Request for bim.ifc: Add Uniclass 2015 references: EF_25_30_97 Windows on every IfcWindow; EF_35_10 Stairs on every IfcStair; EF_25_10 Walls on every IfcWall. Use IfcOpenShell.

First a look at what the model holds.

```python
import ifcopenshell

model = ifcopenshell.open("bim.ifc")
print(model.schema)
print("classifications:", [c.Name for c in model.by_type("IfcClassification")])
for ifc_class in ("IfcDoor", "IfcRoof", "IfcStair", "IfcWall", "IfcWindow"):
    print(ifc_class, len(model.by_type(ifc_class)))
```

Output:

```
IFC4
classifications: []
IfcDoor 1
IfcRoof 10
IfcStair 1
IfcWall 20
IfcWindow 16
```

```python
import ifcopenshell
import ifcopenshell.api.classification

model = ifcopenshell.open("bim.ifc")

system = ifcopenshell.api.classification.add_classification(model, classification="Uniclass 2015")

codes = {
    "IfcWindow": ("EF_25_30_97", "Windows"),
    "IfcStair": ("EF_35_10", "Stairs"),
    "IfcWall": ("EF_25_10", "Walls"),
}
for ifc_class, (code, name) in codes.items():
    products = model.by_type(ifc_class)
    ifcopenshell.api.classification.add_reference(
        model, products=products, classification=system, identification=code, name=name
    )
    print(code, len(products))

model.write("bim_updated.ifc")
```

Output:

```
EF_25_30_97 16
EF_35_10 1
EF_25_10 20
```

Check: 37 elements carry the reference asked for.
